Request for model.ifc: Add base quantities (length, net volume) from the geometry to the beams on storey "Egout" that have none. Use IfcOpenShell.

First a look at what the model holds.

```python
import ifcopenshell
import ifcopenshell.util.element
import ifcopenshell.util.unit

model = ifcopenshell.open("model.ifc")
print(model.schema)
for unit_type in ("LENGTHUNIT", "AREAUNIT", "VOLUMEUNIT"):
    print(unit_type, ifcopenshell.util.unit.calculate_unit_scale(model, unit_type))
storey = next(s for s in model.by_type("IfcBuildingStorey") if s.Name == "Egout")
beams = [e for e in ifcopenshell.util.element.get_decomposition(storey) if e.is_a("IfcBeam")]
for e in sorted(beams, key=lambda e: e.id()):
    print(e.id(), e.is_a(), e.Name, list(ifcopenshell.util.element.get_psets(e, qtos_only=True)), sep=" | ")
```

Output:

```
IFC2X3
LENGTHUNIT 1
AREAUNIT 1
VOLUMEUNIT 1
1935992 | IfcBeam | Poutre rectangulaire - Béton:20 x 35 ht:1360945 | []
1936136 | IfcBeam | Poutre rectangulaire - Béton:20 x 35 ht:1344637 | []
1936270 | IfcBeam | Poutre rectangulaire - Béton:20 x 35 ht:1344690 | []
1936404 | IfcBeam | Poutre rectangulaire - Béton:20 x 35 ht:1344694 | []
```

```python
import ifcopenshell
import ifcopenshell.api.pset
import ifcopenshell.geom
import ifcopenshell.util.element
import ifcopenshell.util.shape
import ifcopenshell.util.unit

model = ifcopenshell.open("model.ifc")
unit_scale = ifcopenshell.util.unit.calculate_unit_scale(model)
volume_scale = ifcopenshell.util.unit.calculate_unit_scale(model, "VOLUMEUNIT")
settings = ifcopenshell.geom.settings()

storey = next(s for s in model.by_type("IfcBuildingStorey") if s.Name == "Egout")
beams = [e for e in ifcopenshell.util.element.get_decomposition(storey) if e.is_a("IfcBeam")]

for e in sorted(beams, key=lambda e: e.id()):
    if ifcopenshell.util.element.get_psets(e, qtos_only=True, should_inherit=False):
        continue
    # Geometry comes back in metres, in the element's own axes.
    shape = ifcopenshell.geom.create_shape(settings, e)
    values = {
        "Length": ifcopenshell.util.shape.get_max_xyz(shape.geometry) / unit_scale,
        "NetVolume": ifcopenshell.util.shape.get_volume(shape.geometry) / volume_scale,
    }
    qto = ifcopenshell.api.pset.add_qto(model, product=e, name="BaseQuantities")
    ifcopenshell.api.pset.edit_qto(model, qto=qto, properties=values)
    print(e.id(), {k: round(v, 3) for k, v in values.items()})

model.write("model_v2.ifc")
```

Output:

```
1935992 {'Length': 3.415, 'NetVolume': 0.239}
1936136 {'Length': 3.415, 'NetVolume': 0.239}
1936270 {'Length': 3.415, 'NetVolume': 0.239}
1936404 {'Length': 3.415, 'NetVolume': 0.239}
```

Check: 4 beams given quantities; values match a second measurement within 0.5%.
